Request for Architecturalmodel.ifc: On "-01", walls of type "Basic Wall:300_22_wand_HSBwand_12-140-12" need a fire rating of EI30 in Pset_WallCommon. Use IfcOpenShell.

First a look at what the model holds.

```python
import ifcopenshell
import ifcopenshell.util.element

model = ifcopenshell.open("Architecturalmodel.ifc")
print(model.schema)
storey = next(s for s in model.by_type("IfcBuildingStorey") if s.Name == "-01")
walls = [e for e in ifcopenshell.util.element.get_decomposition(storey) if e.is_a("IfcWall")]
seen = {}
for e in walls:
    element_type = ifcopenshell.util.element.get_type(e)
    key = (element_type.Name if element_type != e and element_type else None, ifcopenshell.util.element.get_pset(e, "Pset_WallCommon", "FireRating"))
    seen[key] = seen.get(key, 0) + 1
for (name, value), count in sorted(seen.items(), key=str):
    print(count, "x", name, "|", value)
```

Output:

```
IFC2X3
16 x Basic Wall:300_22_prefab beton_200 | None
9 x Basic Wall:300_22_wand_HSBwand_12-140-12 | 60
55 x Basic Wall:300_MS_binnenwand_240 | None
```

```python
import ifcopenshell
import ifcopenshell.api.pset
import ifcopenshell.util.element

model = ifcopenshell.open("Architecturalmodel.ifc")

storey = next(s for s in model.by_type("IfcBuildingStorey") if s.Name == "-01")
walls = [e for e in ifcopenshell.util.element.get_decomposition(storey) if e.is_a("IfcWall")]

count = 0
for e in walls:
    element_type = ifcopenshell.util.element.get_type(e)
    if element_type in (None, e) or element_type.Name != "Basic Wall:300_22_wand_HSBwand_12-140-12":
        continue
    # add_pset returns the element's existing set when there is one.
    pset = ifcopenshell.api.pset.add_pset(model, product=e, name="Pset_WallCommon")
    ifcopenshell.api.pset.edit_pset(model, pset=pset, properties={"FireRating": "EI30"})
    count += 1

print(count, "walls updated")

model.write("Architecturalmodel_edited.ifc")
```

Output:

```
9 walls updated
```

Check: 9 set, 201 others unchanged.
